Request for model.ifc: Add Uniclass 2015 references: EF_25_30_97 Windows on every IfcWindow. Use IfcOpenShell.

First a look at what the model holds.

```python
import ifcopenshell

model = ifcopenshell.open("model.ifc")
print(model.schema)
print("classifications:", [c.Name for c in model.by_type("IfcClassification")])
for ifc_class in ("IfcDoor", "IfcRoof", "IfcStair", "IfcWall", "IfcWindow"):
    print(ifc_class, len(model.by_type(ifc_class)))
```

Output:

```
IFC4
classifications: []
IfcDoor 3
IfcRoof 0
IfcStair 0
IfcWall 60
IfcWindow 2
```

```python
import ifcopenshell
import ifcopenshell.api.classification

model = ifcopenshell.open("model.ifc")

system = ifcopenshell.api.classification.add_classification(model, classification="Uniclass 2015")

codes = {
    "IfcWindow": ("EF_25_30_97", "Windows"),
}
for ifc_class, (code, name) in codes.items():
    products = model.by_type(ifc_class)
    ifcopenshell.api.classification.add_reference(
        model, products=products, classification=system, identification=code, name=name
    )
    print(code, len(products))

model.write("model_v2.ifc")
```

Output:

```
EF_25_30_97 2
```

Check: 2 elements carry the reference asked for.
